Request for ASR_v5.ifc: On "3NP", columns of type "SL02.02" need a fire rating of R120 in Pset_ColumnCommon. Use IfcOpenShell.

First a look at what the model holds.

```python
import ifcopenshell
import ifcopenshell.util.element

model = ifcopenshell.open("ASR_v5.ifc")
print(model.schema)
storey = next(s for s in model.by_type("IfcBuildingStorey") if s.Name == "3NP")
columns = [e for e in ifcopenshell.util.element.get_decomposition(storey) if e.is_a("IfcColumn")]
seen = {}
for e in columns:
    element_type = ifcopenshell.util.element.get_type(e)
    key = (element_type.Name if element_type != e and element_type else None, ifcopenshell.util.element.get_pset(e, "Pset_ColumnCommon", "FireRating"))
    seen[key] = seen.get(key, 0) + 1
for (name, value), count in sorted(seen.items(), key=str):
    print(count, "x", name, "|", value)
```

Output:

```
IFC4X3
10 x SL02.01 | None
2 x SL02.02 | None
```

```python
import ifcopenshell
import ifcopenshell.api.pset
import ifcopenshell.util.element

model = ifcopenshell.open("ASR_v5.ifc")

storey = next(s for s in model.by_type("IfcBuildingStorey") if s.Name == "3NP")
columns = [e for e in ifcopenshell.util.element.get_decomposition(storey) if e.is_a("IfcColumn")]

count = 0
for e in columns:
    element_type = ifcopenshell.util.element.get_type(e)
    if element_type in (None, e) or element_type.Name != "SL02.02":
        continue
    # add_pset returns the element's existing set when there is one.
    pset = ifcopenshell.api.pset.add_pset(model, product=e, name="Pset_ColumnCommon")
    ifcopenshell.api.pset.edit_pset(model, pset=pset, properties={"FireRating": "R120"})
    count += 1

print(count, "columns updated")

model.write("ASR_v5_v2.ifc")
```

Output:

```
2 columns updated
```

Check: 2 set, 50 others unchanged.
